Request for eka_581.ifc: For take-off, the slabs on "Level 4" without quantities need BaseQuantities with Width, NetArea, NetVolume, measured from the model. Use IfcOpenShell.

First a look at what the model holds.

```python
import ifcopenshell
import ifcopenshell.util.element
import ifcopenshell.util.unit

model = ifcopenshell.open("eka_581.ifc")
print(model.schema)
for unit_type in ("LENGTHUNIT", "AREAUNIT", "VOLUMEUNIT"):
    print(unit_type, ifcopenshell.util.unit.calculate_unit_scale(model, unit_type))
storey = next(s for s in model.by_type("IfcBuildingStorey") if s.Name == "Level 4")
slabs = [e for e in ifcopenshell.util.element.get_decomposition(storey) if e.is_a("IfcSlab")]
for e in sorted(slabs, key=lambda e: e.id()):
    print(e.id(), e.is_a(), e.Name, list(ifcopenshell.util.element.get_psets(e, qtos_only=True)), sep=" | ")
```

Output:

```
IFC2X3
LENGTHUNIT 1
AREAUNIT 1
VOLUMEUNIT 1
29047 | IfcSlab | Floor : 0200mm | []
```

```python
import ifcopenshell
import ifcopenshell.api.pset
import ifcopenshell.geom
import ifcopenshell.util.element
import ifcopenshell.util.shape
import ifcopenshell.util.unit

model = ifcopenshell.open("eka_581.ifc")
unit_scale = ifcopenshell.util.unit.calculate_unit_scale(model)
area_scale = ifcopenshell.util.unit.calculate_unit_scale(model, "AREAUNIT")
volume_scale = ifcopenshell.util.unit.calculate_unit_scale(model, "VOLUMEUNIT")
settings = ifcopenshell.geom.settings()

storey = next(s for s in model.by_type("IfcBuildingStorey") if s.Name == "Level 4")
slabs = [e for e in ifcopenshell.util.element.get_decomposition(storey) if e.is_a("IfcSlab")]

for e in sorted(slabs, key=lambda e: e.id()):
    if ifcopenshell.util.element.get_psets(e, qtos_only=True, should_inherit=False):
        continue
    # Geometry comes back in metres, in the element's own axes.
    shape = ifcopenshell.geom.create_shape(settings, e)
    values = {
        "Width": ifcopenshell.util.shape.get_z(shape.geometry) / unit_scale,
        "NetArea": ifcopenshell.util.shape.get_footprint_area(shape.geometry) / area_scale,
        "NetVolume": ifcopenshell.util.shape.get_volume(shape.geometry) / volume_scale,
    }
    qto = ifcopenshell.api.pset.add_qto(model, product=e, name="BaseQuantities")
    ifcopenshell.api.pset.edit_qto(model, qto=qto, properties=values)
    print(e.id(), {k: round(v, 3) for k, v in values.items()})

model.write("eka_581_rev.ifc")
```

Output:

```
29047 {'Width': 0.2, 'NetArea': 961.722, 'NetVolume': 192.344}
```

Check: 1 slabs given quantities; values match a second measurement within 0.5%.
